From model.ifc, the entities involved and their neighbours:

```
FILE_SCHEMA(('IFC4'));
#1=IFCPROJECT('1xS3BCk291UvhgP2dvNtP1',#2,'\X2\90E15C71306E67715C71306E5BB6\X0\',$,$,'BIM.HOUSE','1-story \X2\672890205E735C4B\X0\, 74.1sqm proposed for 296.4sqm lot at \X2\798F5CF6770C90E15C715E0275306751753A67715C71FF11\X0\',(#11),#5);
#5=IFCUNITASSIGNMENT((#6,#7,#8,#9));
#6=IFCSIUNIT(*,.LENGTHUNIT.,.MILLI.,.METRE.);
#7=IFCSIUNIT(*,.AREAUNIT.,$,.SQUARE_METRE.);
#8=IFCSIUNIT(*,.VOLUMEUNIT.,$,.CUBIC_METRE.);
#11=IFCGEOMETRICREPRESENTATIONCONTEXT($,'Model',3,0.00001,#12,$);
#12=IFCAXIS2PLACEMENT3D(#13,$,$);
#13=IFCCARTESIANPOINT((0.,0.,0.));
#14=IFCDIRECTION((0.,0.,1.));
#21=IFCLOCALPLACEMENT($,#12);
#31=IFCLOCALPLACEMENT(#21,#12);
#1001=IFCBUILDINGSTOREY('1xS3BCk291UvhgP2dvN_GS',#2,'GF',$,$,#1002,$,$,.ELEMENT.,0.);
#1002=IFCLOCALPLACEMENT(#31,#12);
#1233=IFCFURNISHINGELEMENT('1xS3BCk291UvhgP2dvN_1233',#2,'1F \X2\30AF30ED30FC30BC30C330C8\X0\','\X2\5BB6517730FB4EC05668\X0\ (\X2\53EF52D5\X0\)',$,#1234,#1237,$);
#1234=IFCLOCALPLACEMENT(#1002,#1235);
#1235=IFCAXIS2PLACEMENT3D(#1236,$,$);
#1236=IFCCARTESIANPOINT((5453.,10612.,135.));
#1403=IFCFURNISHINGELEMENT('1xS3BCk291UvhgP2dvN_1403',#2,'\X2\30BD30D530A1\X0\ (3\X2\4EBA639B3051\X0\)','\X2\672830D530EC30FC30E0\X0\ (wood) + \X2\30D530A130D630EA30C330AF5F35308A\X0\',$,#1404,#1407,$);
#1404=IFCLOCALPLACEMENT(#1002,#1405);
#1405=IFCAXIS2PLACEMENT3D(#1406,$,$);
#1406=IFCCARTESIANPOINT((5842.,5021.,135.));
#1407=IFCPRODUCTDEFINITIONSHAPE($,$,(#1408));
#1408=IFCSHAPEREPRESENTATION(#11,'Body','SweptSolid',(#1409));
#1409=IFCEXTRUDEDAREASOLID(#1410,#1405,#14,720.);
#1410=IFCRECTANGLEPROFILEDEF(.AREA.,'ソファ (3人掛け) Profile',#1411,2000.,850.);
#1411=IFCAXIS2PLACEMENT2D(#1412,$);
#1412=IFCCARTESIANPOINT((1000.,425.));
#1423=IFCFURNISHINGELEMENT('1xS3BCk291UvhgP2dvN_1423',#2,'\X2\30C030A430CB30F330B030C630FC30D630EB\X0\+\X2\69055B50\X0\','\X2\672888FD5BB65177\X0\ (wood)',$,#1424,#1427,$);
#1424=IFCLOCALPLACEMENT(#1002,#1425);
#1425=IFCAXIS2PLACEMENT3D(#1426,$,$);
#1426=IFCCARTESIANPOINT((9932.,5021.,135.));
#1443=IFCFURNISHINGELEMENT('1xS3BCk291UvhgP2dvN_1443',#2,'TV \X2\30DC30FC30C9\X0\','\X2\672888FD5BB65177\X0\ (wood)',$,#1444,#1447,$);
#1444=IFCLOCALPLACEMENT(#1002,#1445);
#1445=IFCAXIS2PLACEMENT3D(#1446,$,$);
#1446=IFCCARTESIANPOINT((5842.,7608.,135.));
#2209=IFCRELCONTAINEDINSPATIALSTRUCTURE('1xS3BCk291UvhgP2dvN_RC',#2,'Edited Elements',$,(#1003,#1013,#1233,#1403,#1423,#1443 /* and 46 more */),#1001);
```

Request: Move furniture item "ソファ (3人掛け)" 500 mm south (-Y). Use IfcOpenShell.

```python
import ifcopenshell
import ifcopenshell.api.geometry
import ifcopenshell.util.placement
import ifcopenshell.util.unit

model = ifcopenshell.open("model.ifc")
unit_scale = ifcopenshell.util.unit.calculate_unit_scale(model)

item = model.by_id(1403)
matrix = ifcopenshell.util.placement.get_local_placement(item.ObjectPlacement)
matrix[1, 3] -= 0.5 / unit_scale
ifcopenshell.api.geometry.edit_object_placement(model, product=item, matrix=matrix, is_si=False)

print(ifcopenshell.util.placement.get_local_placement(item.ObjectPlacement).round(3) + 0.0)

model.write("model_updated.ifc")
```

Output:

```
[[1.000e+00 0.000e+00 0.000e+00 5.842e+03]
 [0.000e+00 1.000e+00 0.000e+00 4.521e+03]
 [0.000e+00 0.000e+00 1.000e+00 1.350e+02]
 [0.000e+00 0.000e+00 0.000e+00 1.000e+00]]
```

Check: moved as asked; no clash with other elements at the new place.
